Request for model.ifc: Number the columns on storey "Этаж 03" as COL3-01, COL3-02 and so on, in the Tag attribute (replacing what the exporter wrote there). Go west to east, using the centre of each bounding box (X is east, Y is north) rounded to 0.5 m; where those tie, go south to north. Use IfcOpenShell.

First a look at what the model holds.

```python
import ifcopenshell
import ifcopenshell.util.element
import ifcopenshell.util.placement

model = ifcopenshell.open("model.ifc")
print(model.schema)
storey = next(s for s in model.by_type("IfcBuildingStorey") if s.Name == "Этаж 03")
columns = [e for e in ifcopenshell.util.element.get_decomposition(storey) if e.is_a("IfcColumn")]
for e in sorted(columns, key=lambda e: e.id()):
    origin = ifcopenshell.util.placement.get_local_placement(e.ObjectPlacement)[:3, 3]
    print(e.id(), e.Tag, e.Name, origin.round(2) + 0.0, sep=" | ")
```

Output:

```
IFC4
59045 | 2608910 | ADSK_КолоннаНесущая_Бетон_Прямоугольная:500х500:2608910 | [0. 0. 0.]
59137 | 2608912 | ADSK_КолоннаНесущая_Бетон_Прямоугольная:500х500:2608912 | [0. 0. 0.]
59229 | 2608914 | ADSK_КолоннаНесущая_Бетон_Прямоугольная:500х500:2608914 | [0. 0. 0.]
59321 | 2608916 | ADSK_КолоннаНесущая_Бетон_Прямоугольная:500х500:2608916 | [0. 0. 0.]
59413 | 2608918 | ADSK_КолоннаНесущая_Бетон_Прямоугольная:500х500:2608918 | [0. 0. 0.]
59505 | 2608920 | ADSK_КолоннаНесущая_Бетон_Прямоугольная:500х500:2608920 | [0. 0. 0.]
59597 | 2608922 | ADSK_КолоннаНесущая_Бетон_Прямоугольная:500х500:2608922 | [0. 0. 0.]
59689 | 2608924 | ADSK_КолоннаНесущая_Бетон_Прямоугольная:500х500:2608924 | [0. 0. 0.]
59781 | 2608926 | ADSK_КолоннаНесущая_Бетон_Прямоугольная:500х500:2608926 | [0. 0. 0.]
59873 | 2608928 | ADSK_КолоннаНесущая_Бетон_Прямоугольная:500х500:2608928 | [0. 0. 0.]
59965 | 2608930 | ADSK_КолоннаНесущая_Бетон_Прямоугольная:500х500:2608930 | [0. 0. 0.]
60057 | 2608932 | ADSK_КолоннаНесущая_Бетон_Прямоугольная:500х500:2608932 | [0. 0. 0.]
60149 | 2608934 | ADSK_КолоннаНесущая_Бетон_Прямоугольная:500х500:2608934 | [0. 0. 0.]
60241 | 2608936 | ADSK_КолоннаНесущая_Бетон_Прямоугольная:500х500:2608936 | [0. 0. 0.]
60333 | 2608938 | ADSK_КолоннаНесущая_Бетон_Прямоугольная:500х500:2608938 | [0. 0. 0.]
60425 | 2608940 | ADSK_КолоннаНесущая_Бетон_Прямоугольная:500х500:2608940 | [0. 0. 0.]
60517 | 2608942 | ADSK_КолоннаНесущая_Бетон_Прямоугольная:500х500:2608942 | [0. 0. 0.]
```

```python
import ifcopenshell
import ifcopenshell.geom
import ifcopenshell.util.element
import ifcopenshell.util.shape

model = ifcopenshell.open("model.ifc")
settings = ifcopenshell.geom.settings()
settings.set("use-world-coords", True)


def centre(element):
    shape = ifcopenshell.geom.create_shape(settings, element)
    return ifcopenshell.util.shape.get_bbox_centroid(shape.geometry)


storey = next(s for s in model.by_type("IfcBuildingStorey") if s.Name == "Этаж 03")
columns = [e for e in ifcopenshell.util.element.get_decomposition(storey) if e.is_a("IfcColumn")]

# Insertion points can sit at a corner or the storey origin, so sort by the geometry (in metres).
centres = {e: centre(e) for e in columns}
columns.sort(key=lambda e: (round(centres[e][0] / 0.5), centres[e][1]))

for i, e in enumerate(columns, start=1):
    number = f"COL3-{i:02d}"
    e.Tag = number
    print(e.id(), number)

model.write("model_rev.ifc")
```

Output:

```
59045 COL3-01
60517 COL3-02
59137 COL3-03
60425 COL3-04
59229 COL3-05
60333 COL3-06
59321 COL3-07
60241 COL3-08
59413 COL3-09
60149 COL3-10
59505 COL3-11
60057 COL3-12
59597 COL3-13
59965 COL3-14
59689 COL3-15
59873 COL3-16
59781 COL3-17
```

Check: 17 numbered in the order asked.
